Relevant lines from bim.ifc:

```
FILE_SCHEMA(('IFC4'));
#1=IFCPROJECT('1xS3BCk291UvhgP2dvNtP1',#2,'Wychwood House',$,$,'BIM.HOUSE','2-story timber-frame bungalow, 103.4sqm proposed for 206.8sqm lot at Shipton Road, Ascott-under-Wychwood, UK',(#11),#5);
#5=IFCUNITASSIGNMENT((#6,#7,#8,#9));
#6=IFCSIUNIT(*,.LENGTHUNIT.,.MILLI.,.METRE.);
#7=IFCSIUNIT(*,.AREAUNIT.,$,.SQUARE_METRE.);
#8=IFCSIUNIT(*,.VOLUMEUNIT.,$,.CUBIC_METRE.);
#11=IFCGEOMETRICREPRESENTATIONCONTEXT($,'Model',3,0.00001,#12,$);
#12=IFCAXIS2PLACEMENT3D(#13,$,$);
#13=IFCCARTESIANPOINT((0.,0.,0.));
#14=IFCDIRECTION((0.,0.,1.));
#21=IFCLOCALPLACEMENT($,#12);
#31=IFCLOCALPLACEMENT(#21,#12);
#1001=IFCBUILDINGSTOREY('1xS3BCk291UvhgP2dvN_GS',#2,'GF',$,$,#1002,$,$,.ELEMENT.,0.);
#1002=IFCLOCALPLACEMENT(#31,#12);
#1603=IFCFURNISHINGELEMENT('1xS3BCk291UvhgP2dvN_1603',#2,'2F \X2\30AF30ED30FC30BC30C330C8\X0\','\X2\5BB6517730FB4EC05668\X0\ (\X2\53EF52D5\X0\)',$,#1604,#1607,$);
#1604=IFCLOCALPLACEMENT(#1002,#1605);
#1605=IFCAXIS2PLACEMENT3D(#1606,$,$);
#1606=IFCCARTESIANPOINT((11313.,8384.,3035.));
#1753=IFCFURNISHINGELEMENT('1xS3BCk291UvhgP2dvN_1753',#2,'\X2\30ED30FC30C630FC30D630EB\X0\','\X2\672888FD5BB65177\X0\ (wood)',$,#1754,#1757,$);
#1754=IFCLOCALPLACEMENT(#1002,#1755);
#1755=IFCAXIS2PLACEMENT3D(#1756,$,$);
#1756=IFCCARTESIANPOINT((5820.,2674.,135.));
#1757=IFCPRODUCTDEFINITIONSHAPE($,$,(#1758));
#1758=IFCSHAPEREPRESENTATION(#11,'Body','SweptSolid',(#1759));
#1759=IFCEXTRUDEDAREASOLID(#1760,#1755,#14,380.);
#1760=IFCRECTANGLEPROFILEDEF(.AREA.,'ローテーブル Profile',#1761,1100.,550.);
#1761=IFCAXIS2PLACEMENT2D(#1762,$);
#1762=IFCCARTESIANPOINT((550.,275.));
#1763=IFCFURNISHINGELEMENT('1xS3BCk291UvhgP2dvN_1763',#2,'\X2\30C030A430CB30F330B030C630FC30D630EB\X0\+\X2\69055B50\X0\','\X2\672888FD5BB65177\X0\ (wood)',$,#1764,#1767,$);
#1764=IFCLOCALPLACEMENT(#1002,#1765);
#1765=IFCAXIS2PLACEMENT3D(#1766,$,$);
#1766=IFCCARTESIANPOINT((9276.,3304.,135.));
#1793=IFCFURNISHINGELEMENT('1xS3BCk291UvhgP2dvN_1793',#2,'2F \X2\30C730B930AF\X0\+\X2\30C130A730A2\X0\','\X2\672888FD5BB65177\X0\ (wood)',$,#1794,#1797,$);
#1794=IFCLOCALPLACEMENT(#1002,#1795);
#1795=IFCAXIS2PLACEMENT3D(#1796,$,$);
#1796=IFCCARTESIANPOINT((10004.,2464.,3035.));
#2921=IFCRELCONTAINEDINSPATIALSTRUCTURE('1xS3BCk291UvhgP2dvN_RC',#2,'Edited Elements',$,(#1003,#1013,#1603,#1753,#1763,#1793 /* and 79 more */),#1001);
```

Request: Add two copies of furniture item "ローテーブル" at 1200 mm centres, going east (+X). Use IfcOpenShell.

```python
import numpy as np
import ifcopenshell
import ifcopenshell.api.geometry
import ifcopenshell.api.root
import ifcopenshell.util.element
import ifcopenshell.util.placement
import ifcopenshell.util.unit

model = ifcopenshell.open("bim.ifc")
unit_scale = ifcopenshell.util.unit.calculate_unit_scale(model)


def reuse_history(source, copy):
    """copy_class also copies each property set's owner history, people and application; keep the originals."""
    for rel in copy.IsDefinedBy:
        if rel.is_a("IfcRelDefinesByProperties") and (history := rel.RelatingPropertyDefinition.OwnerHistory):
            rel.RelatingPropertyDefinition.OwnerHistory = source.OwnerHistory
            ifcopenshell.util.element.remove_deep2(model, history)


source = model.by_guid("1xS3BCk291UvhgP2dvN_1753")
base = ifcopenshell.util.placement.get_local_placement(source.ObjectPlacement)
step = np.array([1.0, 0.0, 0.0]) * 1.2 / unit_scale

for i in range(1, 3):
    copy = ifcopenshell.api.root.copy_class(model, product=source)
    copy.Representation = ifcopenshell.util.element.copy_deep(
        model, source.Representation, exclude=["IfcGeometricRepresentationContext", "IfcRepresentationMap"]
    )
    reuse_history(source, copy)
    matrix = base.copy()
    matrix[:3, 3] += i * step
    print("added at", matrix[:3, 3].round(3) + 0.0)
    ifcopenshell.api.geometry.edit_object_placement(model, product=copy, matrix=matrix, is_si=False)

model.write("bim_rev.ifc")
```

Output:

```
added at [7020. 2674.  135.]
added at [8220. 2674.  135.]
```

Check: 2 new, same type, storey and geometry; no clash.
